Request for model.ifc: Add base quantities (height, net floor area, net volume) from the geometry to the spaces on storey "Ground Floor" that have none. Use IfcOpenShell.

First a look at what the model holds.

```python
import ifcopenshell
import ifcopenshell.util.element
import ifcopenshell.util.unit

model = ifcopenshell.open("model.ifc")
print(model.schema)
for unit_type in ("LENGTHUNIT", "AREAUNIT", "VOLUMEUNIT"):
    print(unit_type, ifcopenshell.util.unit.calculate_unit_scale(model, unit_type))
storey = next(s for s in model.by_type("IfcBuildingStorey") if s.Name == "Ground Floor")
spaces = [e for e in ifcopenshell.util.element.get_decomposition(storey) if e.is_a("IfcSpace")]
for e in sorted(spaces, key=lambda e: e.id()):
    print(e.id(), e.is_a(), e.Name, list(ifcopenshell.util.element.get_psets(e, qtos_only=True)), sep=" | ")
```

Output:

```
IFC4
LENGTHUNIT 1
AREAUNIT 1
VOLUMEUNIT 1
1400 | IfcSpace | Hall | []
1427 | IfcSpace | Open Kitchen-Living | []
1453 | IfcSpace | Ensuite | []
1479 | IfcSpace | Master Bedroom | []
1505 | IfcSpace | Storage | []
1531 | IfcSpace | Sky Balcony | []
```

```python
import ifcopenshell
import ifcopenshell.api.pset
import ifcopenshell.geom
import ifcopenshell.util.element
import ifcopenshell.util.shape
import ifcopenshell.util.unit

model = ifcopenshell.open("model.ifc")
unit_scale = ifcopenshell.util.unit.calculate_unit_scale(model)
area_scale = ifcopenshell.util.unit.calculate_unit_scale(model, "AREAUNIT")
volume_scale = ifcopenshell.util.unit.calculate_unit_scale(model, "VOLUMEUNIT")
settings = ifcopenshell.geom.settings()

storey = next(s for s in model.by_type("IfcBuildingStorey") if s.Name == "Ground Floor")
spaces = [e for e in ifcopenshell.util.element.get_decomposition(storey) if e.is_a("IfcSpace")]

for e in sorted(spaces, key=lambda e: e.id()):
    if ifcopenshell.util.element.get_psets(e, qtos_only=True, should_inherit=False):
        continue
    # Geometry comes back in metres, in the element's own axes.
    shape = ifcopenshell.geom.create_shape(settings, e)
    values = {
        "Height": ifcopenshell.util.shape.get_z(shape.geometry) / unit_scale,
        "NetFloorArea": ifcopenshell.util.shape.get_footprint_area(shape.geometry) / area_scale,
        "NetVolume": ifcopenshell.util.shape.get_volume(shape.geometry) / volume_scale,
    }
    qto = ifcopenshell.api.pset.add_qto(model, product=e, name="Qto_SpaceBaseQuantities")
    ifcopenshell.api.pset.edit_qto(model, qto=qto, properties=values)
    print(e.id(), {k: round(v, 3) for k, v in values.items()})

model.write("model-out.ifc")
```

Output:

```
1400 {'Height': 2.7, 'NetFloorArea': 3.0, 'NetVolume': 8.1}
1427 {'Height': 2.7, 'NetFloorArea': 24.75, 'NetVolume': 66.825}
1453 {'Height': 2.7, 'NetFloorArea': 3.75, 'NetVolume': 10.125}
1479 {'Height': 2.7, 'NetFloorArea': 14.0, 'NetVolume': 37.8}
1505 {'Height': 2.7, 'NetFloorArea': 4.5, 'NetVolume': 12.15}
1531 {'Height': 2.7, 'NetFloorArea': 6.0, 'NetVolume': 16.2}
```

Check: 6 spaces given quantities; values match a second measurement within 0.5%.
